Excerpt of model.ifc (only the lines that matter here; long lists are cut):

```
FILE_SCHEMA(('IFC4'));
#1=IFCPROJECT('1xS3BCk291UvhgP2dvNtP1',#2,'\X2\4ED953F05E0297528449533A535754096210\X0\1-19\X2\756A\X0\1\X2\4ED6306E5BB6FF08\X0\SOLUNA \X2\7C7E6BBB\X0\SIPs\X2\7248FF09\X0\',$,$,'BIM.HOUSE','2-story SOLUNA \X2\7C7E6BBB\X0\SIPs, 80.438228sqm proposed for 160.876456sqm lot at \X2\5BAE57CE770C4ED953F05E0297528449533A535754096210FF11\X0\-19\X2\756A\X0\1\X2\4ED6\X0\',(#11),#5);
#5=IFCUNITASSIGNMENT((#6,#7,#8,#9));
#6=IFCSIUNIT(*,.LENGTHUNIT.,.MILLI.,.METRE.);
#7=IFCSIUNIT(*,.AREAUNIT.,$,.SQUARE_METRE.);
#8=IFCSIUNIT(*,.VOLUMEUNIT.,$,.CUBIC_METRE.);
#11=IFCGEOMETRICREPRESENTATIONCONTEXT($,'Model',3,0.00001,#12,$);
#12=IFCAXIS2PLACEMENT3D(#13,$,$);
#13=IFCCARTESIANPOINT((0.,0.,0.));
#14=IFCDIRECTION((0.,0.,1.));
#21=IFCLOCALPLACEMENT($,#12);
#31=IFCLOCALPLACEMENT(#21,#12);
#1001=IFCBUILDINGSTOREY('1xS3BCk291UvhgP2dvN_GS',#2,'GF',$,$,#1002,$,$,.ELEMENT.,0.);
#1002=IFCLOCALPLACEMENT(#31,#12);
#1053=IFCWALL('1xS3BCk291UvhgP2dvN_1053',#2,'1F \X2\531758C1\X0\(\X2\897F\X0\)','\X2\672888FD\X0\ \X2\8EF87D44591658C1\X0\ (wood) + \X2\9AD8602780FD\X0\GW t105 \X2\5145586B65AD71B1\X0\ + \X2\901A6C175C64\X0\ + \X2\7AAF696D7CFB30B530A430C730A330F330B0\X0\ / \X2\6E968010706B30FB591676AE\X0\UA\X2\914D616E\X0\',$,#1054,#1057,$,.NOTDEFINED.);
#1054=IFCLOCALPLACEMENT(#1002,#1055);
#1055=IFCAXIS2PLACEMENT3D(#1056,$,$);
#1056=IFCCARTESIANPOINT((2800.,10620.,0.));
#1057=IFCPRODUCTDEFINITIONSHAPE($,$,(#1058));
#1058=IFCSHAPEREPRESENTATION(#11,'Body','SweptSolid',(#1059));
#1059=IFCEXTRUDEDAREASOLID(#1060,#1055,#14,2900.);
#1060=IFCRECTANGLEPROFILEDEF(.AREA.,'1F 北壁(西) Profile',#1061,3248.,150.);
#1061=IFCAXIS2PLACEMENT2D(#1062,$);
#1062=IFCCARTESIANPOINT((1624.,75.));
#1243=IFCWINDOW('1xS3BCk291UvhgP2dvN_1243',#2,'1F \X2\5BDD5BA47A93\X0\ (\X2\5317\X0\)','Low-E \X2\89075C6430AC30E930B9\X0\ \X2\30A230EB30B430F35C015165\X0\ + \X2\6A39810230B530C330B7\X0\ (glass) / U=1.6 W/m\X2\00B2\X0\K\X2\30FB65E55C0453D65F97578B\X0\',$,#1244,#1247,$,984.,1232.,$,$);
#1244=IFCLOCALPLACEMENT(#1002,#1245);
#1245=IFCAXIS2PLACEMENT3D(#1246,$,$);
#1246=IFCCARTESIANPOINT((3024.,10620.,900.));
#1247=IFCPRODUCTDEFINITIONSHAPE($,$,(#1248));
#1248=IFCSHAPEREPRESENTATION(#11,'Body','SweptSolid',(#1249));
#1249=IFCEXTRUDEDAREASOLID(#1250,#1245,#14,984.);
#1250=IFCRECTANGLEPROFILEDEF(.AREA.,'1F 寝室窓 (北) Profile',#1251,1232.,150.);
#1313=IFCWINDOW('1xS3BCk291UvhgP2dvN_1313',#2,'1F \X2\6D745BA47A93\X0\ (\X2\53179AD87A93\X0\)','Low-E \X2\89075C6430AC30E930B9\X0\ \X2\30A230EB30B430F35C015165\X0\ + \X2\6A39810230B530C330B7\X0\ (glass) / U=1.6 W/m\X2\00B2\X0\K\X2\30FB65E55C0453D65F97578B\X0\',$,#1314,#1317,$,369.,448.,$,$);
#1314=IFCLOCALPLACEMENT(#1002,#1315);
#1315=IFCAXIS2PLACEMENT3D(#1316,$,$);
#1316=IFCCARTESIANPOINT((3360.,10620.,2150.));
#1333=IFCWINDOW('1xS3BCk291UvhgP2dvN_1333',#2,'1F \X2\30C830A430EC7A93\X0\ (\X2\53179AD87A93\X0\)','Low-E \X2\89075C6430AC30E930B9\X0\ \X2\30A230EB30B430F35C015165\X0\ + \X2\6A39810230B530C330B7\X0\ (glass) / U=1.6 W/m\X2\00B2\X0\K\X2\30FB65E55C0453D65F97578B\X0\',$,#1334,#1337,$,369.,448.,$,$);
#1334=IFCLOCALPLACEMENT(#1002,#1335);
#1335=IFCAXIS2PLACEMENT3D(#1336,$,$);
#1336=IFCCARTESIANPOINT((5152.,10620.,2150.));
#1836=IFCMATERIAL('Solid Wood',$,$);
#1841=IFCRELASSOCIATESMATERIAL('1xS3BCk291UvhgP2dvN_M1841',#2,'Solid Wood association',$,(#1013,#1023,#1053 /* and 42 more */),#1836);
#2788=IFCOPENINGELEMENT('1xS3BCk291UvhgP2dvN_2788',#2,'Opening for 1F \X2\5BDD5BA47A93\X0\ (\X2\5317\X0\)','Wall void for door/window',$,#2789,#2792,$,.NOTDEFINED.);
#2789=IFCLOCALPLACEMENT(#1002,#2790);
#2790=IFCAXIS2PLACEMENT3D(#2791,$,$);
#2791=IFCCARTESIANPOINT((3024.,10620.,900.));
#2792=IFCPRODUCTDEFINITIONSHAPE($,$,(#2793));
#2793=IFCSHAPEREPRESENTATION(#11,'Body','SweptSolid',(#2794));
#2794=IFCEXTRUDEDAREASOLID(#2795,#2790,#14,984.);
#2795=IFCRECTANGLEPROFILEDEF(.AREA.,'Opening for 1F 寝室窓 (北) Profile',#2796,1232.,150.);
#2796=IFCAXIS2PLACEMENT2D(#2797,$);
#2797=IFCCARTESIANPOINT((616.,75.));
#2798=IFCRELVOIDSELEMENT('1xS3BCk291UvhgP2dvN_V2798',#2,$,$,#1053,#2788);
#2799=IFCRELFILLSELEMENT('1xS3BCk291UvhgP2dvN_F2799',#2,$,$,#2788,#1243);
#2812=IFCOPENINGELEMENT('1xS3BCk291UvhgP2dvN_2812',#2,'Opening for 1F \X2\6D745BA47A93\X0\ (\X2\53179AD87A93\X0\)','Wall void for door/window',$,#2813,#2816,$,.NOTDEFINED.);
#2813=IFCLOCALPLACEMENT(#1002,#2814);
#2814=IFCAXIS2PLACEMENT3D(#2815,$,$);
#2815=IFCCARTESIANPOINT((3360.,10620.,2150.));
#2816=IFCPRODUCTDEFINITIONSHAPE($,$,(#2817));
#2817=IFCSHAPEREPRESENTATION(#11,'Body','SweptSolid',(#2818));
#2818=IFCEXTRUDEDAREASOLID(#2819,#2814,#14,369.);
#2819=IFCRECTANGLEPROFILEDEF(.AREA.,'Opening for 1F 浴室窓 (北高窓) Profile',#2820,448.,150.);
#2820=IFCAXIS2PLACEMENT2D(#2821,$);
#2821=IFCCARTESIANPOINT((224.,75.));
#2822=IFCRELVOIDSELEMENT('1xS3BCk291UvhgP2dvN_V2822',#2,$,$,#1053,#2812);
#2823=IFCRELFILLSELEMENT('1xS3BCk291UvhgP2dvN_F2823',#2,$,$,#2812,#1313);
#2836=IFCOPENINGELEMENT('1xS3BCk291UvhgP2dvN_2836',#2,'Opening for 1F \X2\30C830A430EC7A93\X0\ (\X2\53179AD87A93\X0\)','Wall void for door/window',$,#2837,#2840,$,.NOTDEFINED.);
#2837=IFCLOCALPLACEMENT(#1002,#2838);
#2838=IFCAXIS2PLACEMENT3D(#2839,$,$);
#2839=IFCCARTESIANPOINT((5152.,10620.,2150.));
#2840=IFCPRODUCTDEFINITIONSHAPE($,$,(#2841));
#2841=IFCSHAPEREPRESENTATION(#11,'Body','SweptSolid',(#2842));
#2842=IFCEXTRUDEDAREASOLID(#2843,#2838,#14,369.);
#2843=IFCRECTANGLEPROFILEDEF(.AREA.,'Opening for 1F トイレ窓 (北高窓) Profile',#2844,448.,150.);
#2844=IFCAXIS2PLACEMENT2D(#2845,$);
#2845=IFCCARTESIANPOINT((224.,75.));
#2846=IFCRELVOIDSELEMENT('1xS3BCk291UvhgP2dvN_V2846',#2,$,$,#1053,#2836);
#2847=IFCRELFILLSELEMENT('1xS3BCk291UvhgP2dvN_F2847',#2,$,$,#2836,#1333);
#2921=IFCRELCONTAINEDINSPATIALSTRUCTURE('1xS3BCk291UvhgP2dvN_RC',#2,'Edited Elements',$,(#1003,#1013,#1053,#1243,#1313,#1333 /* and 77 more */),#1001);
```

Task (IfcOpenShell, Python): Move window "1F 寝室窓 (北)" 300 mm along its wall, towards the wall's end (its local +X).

```python
import ifcopenshell
import ifcopenshell.api.geometry
import ifcopenshell.util.placement

model = ifcopenshell.open("model.ifc")

window = model.by_guid("1xS3BCk291UvhgP2dvN_1243")
opening = window.FillsVoids[0].RelatingOpeningElement
wall = opening.VoidsElements[0].RelatingBuildingElement

wall_matrix = ifcopenshell.util.placement.get_local_placement(wall.ObjectPlacement)
shift = wall_matrix[:3, 0] * 300.0
before = ifcopenshell.util.placement.get_local_placement(window.ObjectPlacement)[:3, 3].copy()

# The window is not placed relative to its opening, so move both.
for product in (opening, window):
    matrix = ifcopenshell.util.placement.get_local_placement(product.ObjectPlacement)
    matrix[:3, 3] += shift
    ifcopenshell.api.geometry.edit_object_placement(model, product=product, matrix=matrix, is_si=False)

after = ifcopenshell.util.placement.get_local_placement(window.ObjectPlacement)[:3, 3]
print("window moved by", (after - before).round(3) + 0.0)

model.write("model-out.ifc")
```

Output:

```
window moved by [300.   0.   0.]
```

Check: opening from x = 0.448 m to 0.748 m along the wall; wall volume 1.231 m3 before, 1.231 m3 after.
